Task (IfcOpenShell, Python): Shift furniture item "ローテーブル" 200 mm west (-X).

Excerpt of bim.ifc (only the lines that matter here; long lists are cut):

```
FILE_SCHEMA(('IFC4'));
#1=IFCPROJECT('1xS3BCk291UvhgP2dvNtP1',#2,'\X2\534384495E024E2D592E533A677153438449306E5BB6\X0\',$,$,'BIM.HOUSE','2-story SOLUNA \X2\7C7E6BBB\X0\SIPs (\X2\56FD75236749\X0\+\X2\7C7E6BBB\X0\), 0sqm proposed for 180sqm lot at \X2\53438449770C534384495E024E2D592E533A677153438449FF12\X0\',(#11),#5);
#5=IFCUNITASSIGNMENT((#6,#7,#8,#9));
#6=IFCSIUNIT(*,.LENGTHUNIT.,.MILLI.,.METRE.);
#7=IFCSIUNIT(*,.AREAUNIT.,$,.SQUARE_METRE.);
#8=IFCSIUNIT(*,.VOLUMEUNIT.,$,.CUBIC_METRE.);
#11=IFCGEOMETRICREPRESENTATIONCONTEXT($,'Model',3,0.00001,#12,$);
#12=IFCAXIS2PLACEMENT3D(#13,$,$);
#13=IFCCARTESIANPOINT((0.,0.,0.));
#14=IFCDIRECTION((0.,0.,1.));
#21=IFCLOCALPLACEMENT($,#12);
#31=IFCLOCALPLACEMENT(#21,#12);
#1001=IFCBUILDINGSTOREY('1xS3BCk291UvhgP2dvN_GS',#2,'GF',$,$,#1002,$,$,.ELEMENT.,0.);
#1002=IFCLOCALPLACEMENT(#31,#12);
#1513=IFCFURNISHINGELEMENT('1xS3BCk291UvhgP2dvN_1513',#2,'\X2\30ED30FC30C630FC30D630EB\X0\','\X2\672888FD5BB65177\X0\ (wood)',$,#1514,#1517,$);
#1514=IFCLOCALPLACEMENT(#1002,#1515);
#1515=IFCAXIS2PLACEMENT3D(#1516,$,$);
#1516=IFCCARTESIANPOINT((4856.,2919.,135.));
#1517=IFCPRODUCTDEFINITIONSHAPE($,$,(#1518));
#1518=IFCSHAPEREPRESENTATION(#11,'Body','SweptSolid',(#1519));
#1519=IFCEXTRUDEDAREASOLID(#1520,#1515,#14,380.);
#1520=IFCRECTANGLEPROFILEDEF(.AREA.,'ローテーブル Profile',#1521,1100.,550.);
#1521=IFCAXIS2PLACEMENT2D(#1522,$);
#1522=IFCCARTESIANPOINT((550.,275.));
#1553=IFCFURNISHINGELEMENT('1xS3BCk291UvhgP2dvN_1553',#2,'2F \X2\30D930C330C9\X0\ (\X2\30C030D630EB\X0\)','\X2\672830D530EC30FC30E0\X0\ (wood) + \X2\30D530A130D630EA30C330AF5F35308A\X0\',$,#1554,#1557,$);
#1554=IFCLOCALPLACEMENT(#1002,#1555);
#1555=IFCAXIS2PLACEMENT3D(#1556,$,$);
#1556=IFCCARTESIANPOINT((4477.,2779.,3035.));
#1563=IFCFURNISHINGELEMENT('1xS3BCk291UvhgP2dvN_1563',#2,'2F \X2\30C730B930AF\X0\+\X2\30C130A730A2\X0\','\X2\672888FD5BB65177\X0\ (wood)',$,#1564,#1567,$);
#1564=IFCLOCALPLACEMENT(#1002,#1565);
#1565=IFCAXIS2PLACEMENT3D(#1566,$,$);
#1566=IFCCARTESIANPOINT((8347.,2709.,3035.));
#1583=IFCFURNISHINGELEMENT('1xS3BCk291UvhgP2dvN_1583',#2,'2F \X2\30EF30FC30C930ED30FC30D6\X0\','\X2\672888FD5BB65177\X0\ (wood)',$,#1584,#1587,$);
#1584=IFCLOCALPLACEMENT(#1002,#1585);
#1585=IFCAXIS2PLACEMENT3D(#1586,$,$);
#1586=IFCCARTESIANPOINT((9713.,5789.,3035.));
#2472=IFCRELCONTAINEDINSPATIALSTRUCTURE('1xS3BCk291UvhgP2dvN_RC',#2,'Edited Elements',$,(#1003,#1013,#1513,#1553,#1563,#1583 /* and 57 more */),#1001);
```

```python
import ifcopenshell
import ifcopenshell.api.geometry
import ifcopenshell.util.placement

model = ifcopenshell.open("bim.ifc")

item = model.by_guid("1xS3BCk291UvhgP2dvN_1513")
matrix = ifcopenshell.util.placement.get_local_placement(item.ObjectPlacement)
matrix[0, 3] -= 200.0
ifcopenshell.api.geometry.edit_object_placement(model, product=item, matrix=matrix, is_si=False)

print(ifcopenshell.util.placement.get_local_placement(item.ObjectPlacement).round(3) + 0.0)

model.write("bim-out.ifc")
```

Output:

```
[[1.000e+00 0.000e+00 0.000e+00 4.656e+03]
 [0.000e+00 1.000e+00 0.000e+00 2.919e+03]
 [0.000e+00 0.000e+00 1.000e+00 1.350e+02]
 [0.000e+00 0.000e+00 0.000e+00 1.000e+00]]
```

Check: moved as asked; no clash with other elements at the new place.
